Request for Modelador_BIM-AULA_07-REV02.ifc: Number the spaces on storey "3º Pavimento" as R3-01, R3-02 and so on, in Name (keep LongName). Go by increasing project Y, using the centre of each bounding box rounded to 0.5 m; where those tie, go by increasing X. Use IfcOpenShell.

First a look at what the model holds.

```python
import ifcopenshell
import ifcopenshell.util.element
import ifcopenshell.util.placement

model = ifcopenshell.open("Modelador_BIM-AULA_07-REV02.ifc")
print(model.schema)
storey = next(s for s in model.by_type("IfcBuildingStorey") if s.Name == "3º Pavimento")
spaces = [e for e in ifcopenshell.util.element.get_decomposition(storey) if e.is_a("IfcSpace")]
for e in sorted(spaces, key=lambda e: e.id()):
    origin = ifcopenshell.util.placement.get_local_placement(e.ObjectPlacement)[:3, 3]
    print(e.id(), e.Name, e.LongName, origin.round(2) + 0.0, sep=" | ")
```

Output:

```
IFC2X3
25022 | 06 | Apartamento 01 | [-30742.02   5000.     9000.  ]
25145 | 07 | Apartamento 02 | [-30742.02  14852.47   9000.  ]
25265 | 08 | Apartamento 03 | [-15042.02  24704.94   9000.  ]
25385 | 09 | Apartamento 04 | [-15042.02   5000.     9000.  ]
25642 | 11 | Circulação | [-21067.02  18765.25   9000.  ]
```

```python
import ifcopenshell
import ifcopenshell.geom
import ifcopenshell.util.element
import ifcopenshell.util.shape

model = ifcopenshell.open("Modelador_BIM-AULA_07-REV02.ifc")
settings = ifcopenshell.geom.settings()
settings.set("use-world-coords", True)


def centre(element):
    shape = ifcopenshell.geom.create_shape(settings, element)
    return ifcopenshell.util.shape.get_bbox_centroid(shape.geometry)


storey = next(s for s in model.by_type("IfcBuildingStorey") if s.Name == "3º Pavimento")
spaces = [e for e in ifcopenshell.util.element.get_decomposition(storey) if e.is_a("IfcSpace")]

# Insertion points can sit at a corner or the storey origin, so sort by the geometry (in metres).
centres = {e: centre(e) for e in spaces}
spaces.sort(key=lambda e: (round(centres[e][1] / 0.5), centres[e][0]))

for i, e in enumerate(spaces, start=1):
    number = f"R3-{i:02d}"
    e.Name = number
    print(e.id(), number)

model.write("Modelador_BIM-AULA_07-REV02_updated.ifc")
```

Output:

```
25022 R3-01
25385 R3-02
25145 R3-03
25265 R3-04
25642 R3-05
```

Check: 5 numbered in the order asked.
